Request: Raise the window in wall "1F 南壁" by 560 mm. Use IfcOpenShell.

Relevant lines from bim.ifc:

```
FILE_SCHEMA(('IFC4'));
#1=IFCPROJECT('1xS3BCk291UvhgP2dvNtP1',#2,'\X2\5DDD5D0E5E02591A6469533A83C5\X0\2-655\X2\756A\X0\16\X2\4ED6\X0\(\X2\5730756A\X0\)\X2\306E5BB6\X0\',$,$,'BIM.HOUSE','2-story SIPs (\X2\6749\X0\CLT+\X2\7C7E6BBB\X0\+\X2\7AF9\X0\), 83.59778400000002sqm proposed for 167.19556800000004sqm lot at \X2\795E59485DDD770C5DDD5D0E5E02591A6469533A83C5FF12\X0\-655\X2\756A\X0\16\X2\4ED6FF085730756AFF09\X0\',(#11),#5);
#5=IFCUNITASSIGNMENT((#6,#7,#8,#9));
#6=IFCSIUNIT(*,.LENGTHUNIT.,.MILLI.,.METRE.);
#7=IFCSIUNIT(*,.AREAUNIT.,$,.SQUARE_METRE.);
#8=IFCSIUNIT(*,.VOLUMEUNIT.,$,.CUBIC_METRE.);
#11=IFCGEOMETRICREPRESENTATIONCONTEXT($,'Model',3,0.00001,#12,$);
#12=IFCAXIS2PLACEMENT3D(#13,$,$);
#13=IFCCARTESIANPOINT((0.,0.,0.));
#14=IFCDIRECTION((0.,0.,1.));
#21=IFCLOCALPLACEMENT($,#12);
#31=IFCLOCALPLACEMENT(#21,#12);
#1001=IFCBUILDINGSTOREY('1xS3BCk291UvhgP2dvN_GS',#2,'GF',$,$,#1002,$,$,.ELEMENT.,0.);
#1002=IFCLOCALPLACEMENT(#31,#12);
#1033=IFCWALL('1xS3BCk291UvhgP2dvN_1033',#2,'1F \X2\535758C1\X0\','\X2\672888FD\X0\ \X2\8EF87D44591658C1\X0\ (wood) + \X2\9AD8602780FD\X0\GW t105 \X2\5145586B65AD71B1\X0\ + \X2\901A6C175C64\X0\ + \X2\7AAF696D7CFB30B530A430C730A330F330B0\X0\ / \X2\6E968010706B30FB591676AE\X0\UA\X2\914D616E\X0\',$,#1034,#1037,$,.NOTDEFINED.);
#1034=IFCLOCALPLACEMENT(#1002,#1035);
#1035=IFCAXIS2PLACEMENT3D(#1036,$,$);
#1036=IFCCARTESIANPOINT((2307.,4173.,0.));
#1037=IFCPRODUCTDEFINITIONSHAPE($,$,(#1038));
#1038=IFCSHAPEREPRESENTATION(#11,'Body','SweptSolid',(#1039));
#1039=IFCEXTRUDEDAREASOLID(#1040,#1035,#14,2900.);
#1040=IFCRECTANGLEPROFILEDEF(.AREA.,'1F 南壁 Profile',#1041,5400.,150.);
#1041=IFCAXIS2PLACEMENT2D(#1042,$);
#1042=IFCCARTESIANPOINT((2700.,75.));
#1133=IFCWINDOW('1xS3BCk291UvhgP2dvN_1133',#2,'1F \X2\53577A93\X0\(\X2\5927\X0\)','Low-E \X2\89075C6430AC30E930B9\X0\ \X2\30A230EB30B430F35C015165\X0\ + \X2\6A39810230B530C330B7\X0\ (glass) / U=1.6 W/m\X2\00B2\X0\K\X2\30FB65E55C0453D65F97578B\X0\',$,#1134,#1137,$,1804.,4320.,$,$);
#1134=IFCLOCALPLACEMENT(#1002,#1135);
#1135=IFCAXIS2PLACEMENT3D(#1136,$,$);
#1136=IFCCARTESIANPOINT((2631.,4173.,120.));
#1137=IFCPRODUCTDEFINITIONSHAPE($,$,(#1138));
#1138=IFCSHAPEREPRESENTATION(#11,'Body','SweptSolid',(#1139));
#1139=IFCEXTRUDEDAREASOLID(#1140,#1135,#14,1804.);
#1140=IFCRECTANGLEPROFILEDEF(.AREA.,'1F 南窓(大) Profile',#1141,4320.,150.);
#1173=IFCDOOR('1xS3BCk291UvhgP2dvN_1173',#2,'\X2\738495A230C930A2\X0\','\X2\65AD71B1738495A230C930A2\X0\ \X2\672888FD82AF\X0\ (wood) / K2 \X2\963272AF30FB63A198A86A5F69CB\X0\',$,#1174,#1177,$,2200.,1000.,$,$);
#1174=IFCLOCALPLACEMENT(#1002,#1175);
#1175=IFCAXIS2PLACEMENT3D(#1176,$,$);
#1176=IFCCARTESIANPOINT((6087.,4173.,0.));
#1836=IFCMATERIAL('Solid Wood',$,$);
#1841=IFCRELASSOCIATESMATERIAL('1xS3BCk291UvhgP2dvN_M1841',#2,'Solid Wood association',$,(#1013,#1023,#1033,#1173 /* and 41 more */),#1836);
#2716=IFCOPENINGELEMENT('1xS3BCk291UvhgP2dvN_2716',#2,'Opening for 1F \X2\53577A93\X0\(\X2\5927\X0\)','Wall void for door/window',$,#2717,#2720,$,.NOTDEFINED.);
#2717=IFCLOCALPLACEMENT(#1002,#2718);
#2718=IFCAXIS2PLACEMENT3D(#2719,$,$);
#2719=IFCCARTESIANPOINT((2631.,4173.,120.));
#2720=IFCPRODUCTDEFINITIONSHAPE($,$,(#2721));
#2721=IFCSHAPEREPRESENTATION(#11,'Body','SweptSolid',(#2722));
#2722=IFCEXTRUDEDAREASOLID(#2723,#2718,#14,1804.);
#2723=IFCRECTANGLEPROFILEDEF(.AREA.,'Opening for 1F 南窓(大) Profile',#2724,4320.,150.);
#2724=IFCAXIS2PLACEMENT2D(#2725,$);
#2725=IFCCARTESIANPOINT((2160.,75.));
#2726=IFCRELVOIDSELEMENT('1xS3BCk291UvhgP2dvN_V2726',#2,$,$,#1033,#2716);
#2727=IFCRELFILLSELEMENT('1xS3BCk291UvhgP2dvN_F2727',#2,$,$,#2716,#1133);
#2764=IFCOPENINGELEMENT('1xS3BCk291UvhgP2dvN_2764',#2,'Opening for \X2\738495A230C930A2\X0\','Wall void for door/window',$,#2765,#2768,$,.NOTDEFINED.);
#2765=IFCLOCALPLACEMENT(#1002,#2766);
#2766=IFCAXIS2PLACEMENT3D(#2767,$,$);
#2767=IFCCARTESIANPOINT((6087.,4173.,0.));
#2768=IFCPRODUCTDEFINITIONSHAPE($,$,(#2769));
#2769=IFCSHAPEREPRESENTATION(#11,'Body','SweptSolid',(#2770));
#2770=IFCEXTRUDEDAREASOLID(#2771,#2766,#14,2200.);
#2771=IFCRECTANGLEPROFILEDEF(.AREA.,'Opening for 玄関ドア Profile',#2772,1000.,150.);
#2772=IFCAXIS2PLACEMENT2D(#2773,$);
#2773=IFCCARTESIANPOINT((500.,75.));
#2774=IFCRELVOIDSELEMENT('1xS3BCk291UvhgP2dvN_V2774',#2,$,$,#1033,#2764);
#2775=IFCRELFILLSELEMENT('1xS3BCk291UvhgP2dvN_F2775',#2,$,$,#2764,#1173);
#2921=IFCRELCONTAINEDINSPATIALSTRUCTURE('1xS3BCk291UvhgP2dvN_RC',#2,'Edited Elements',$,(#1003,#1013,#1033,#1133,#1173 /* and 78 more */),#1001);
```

```python
import numpy as np
import ifcopenshell
import ifcopenshell.api.geometry
import ifcopenshell.util.placement
import ifcopenshell.util.unit

model = ifcopenshell.open("bim.ifc")
unit_scale = ifcopenshell.util.unit.calculate_unit_scale(model)

window = model.by_id(1133)
opening = window.FillsVoids[0].RelatingOpeningElement
dz = 560.0

shift = np.array([0.0, 0.0, dz])
# The window is not placed relative to its opening, so move both.
for product in (opening, window):
    matrix = ifcopenshell.util.placement.get_local_placement(product.ObjectPlacement)
    matrix[:3, 3] += shift
    ifcopenshell.api.geometry.edit_object_placement(model, product=product, matrix=matrix, is_si=False)

print(f"moved by {dz * unit_scale:+.3f} m")

model.write("bim_v2.ifc")
```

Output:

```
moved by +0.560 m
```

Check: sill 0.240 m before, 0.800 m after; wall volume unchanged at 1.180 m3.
